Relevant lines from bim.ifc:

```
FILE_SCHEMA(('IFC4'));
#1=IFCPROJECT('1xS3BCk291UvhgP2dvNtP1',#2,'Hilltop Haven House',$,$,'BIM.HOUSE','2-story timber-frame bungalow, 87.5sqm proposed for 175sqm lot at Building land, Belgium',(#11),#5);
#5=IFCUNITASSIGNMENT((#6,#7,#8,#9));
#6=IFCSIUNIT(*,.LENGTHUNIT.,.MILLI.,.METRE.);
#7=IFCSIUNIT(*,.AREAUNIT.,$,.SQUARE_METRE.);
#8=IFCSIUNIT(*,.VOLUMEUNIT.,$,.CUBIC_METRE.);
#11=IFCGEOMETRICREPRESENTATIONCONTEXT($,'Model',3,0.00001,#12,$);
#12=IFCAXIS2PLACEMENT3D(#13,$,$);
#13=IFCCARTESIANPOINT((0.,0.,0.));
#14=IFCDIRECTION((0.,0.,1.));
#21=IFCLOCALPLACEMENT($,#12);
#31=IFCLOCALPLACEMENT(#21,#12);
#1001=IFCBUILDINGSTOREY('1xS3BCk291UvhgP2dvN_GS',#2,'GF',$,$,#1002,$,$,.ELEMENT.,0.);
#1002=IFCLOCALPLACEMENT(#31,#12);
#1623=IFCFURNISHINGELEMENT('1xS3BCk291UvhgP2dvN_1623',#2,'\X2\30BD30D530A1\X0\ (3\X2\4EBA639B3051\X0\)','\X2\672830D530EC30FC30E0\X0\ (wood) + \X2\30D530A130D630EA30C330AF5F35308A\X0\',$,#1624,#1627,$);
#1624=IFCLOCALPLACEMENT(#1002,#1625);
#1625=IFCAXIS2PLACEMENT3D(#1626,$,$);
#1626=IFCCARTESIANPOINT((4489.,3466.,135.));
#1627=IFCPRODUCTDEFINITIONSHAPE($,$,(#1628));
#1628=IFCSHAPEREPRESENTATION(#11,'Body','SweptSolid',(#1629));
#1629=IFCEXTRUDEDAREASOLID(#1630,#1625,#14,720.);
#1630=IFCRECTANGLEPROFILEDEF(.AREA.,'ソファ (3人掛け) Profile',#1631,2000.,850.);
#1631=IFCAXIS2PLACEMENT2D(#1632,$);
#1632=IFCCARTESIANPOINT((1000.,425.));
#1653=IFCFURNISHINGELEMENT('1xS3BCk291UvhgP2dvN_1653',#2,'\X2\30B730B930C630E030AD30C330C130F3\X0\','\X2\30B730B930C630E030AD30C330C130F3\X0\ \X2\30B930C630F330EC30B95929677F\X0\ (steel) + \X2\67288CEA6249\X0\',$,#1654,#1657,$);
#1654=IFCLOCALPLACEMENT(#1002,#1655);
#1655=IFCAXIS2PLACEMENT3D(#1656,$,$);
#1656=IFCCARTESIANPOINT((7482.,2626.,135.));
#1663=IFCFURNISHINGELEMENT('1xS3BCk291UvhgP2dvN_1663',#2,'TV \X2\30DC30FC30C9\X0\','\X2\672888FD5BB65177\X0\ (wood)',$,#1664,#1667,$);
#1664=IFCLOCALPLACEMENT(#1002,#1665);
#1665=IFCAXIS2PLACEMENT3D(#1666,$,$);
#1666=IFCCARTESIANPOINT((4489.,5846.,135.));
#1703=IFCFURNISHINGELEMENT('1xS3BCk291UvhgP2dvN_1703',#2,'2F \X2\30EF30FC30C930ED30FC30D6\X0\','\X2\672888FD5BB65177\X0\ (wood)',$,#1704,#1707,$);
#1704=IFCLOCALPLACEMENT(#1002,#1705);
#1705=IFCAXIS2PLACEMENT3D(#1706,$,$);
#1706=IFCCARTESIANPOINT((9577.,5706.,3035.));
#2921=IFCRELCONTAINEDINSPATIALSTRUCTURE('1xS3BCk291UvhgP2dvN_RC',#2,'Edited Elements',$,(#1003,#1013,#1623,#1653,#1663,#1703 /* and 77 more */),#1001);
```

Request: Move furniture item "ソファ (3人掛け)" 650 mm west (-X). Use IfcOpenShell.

```python
import ifcopenshell
import ifcopenshell.api.geometry
import ifcopenshell.util.placement
import ifcopenshell.util.unit

model = ifcopenshell.open("bim.ifc")
unit_scale = ifcopenshell.util.unit.calculate_unit_scale(model)

item = model.by_guid("1xS3BCk291UvhgP2dvN_1623")
matrix = ifcopenshell.util.placement.get_local_placement(item.ObjectPlacement)
matrix[0, 3] -= 0.65 / unit_scale
ifcopenshell.api.geometry.edit_object_placement(model, product=item, matrix=matrix, is_si=False)

print(ifcopenshell.util.placement.get_local_placement(item.ObjectPlacement).round(3) + 0.0)

model.write("bim_v2.ifc")
```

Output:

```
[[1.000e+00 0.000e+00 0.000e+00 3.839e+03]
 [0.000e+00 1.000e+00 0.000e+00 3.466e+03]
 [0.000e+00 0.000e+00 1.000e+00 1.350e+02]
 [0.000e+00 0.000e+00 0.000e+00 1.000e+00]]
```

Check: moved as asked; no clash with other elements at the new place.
